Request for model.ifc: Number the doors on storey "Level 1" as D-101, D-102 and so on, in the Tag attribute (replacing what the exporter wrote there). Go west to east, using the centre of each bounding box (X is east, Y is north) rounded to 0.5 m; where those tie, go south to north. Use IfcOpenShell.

First a look at what the model holds.

```python
import ifcopenshell
import ifcopenshell.util.element
import ifcopenshell.util.placement

model = ifcopenshell.open("model.ifc")
print(model.schema)
storey = next(s for s in model.by_type("IfcBuildingStorey") if s.Name == "Level 1")
doors = [e for e in ifcopenshell.util.element.get_decomposition(storey) if e.is_a("IfcDoor")]
for e in sorted(doors, key=lambda e: e.id()):
    origin = ifcopenshell.util.placement.get_local_placement(e.ObjectPlacement)[:3, 3]
    print(e.id(), e.Tag, e.Name, origin.round(2) + 0.0, sep=" | ")
```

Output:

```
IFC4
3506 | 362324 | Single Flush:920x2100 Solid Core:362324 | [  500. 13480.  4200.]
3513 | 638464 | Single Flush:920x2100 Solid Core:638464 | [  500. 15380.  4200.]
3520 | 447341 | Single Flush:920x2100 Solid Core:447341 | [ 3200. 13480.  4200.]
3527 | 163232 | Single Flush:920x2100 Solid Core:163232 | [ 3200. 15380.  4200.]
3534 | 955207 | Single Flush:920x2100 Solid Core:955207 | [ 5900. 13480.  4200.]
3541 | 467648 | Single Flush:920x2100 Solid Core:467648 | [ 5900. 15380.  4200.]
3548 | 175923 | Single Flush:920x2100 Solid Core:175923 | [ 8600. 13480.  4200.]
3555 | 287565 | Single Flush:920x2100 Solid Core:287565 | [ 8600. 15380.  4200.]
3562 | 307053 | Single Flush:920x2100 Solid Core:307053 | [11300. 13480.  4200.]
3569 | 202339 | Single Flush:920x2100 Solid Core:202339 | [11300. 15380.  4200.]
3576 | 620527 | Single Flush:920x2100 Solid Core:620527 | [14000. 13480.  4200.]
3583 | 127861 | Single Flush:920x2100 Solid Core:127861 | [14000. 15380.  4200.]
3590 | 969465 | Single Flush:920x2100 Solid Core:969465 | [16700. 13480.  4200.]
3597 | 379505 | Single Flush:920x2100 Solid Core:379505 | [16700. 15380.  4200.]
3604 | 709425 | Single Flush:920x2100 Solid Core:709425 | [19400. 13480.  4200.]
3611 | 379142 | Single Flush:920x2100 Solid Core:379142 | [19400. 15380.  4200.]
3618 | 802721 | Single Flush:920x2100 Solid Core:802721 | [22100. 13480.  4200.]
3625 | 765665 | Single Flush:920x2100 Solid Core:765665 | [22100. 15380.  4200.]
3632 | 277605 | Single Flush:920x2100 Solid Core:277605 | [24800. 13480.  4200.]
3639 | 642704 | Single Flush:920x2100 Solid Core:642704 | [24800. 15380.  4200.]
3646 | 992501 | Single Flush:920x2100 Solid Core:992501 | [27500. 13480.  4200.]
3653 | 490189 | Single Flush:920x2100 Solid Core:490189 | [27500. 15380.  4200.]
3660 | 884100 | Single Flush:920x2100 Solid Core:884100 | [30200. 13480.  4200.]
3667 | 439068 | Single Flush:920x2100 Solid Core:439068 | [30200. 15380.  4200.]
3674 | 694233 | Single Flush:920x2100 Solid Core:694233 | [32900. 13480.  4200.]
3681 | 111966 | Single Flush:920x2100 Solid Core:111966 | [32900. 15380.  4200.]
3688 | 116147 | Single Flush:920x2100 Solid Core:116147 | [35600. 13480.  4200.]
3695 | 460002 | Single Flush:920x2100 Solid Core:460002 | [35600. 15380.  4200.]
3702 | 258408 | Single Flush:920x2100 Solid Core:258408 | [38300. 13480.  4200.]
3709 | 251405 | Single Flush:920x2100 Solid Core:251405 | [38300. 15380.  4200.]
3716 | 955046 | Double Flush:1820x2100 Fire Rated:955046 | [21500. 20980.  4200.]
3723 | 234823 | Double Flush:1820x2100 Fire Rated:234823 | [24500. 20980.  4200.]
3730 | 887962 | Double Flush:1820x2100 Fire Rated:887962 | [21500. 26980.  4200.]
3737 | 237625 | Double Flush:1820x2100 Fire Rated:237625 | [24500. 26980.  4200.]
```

```python
import ifcopenshell
import ifcopenshell.geom
import ifcopenshell.util.element
import ifcopenshell.util.shape

model = ifcopenshell.open("model.ifc")
settings = ifcopenshell.geom.settings()
settings.set("use-world-coords", True)


def centre(element):
    shape = ifcopenshell.geom.create_shape(settings, element)
    return ifcopenshell.util.shape.get_bbox_centroid(shape.geometry)


storey = next(s for s in model.by_type("IfcBuildingStorey") if s.Name == "Level 1")
doors = [e for e in ifcopenshell.util.element.get_decomposition(storey) if e.is_a("IfcDoor")]

# Insertion points can sit at a corner or the storey origin, so sort by the geometry (in metres).
centres = {e: centre(e) for e in doors}
doors.sort(key=lambda e: (round(centres[e][0] / 0.5), centres[e][1]))

for i, e in enumerate(doors, start=1):
    number = f"D-1{i:02d}"
    e.Tag = number
    print(e.id(), number)

model.write("model_rev.ifc")
```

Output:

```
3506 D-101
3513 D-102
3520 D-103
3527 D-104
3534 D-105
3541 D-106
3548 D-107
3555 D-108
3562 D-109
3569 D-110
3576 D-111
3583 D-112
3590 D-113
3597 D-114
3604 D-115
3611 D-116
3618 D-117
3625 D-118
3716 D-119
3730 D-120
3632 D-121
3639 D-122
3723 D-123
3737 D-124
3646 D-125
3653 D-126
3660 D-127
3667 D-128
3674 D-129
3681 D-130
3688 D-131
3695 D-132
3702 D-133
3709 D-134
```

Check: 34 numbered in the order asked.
